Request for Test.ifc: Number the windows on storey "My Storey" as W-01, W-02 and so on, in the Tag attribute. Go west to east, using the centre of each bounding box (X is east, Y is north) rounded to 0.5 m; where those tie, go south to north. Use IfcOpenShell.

First a look at what the model holds.

```python
import ifcopenshell
import ifcopenshell.util.element
import ifcopenshell.util.placement

model = ifcopenshell.open("Test.ifc")
print(model.schema)
storey = next(s for s in model.by_type("IfcBuildingStorey") if s.Name == "My Storey")
windows = [e for e in ifcopenshell.util.element.get_decomposition(storey) if e.is_a("IfcWindow")]
for e in sorted(windows, key=lambda e: e.id()):
    origin = ifcopenshell.util.placement.get_local_placement(e.ObjectPlacement)[:3, 3]
    print(e.id(), e.Tag, e.Name, origin.round(2) + 0.0, sep=" | ")
```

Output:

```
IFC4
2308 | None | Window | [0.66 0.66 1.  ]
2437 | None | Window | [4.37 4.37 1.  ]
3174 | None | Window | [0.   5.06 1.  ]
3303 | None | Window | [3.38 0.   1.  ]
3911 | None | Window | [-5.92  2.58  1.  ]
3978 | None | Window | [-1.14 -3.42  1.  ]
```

```python
import ifcopenshell
import ifcopenshell.geom
import ifcopenshell.util.element
import ifcopenshell.util.shape

model = ifcopenshell.open("Test.ifc")
settings = ifcopenshell.geom.settings()
settings.set("use-world-coords", True)


def centre(element):
    shape = ifcopenshell.geom.create_shape(settings, element)
    return ifcopenshell.util.shape.get_bbox_centroid(shape.geometry)


storey = next(s for s in model.by_type("IfcBuildingStorey") if s.Name == "My Storey")
windows = [e for e in ifcopenshell.util.element.get_decomposition(storey) if e.is_a("IfcWindow")]

# Insertion points can sit at a corner or the storey origin, so sort by the geometry (in metres).
centres = {e: centre(e) for e in windows}
windows.sort(key=lambda e: (round(centres[e][0] / 0.5), centres[e][1]))

for i, e in enumerate(windows, start=1):
    number = f"W-{i:02d}"
    e.Tag = number
    print(e.id(), number)

model.write("Test_edited.ifc")
```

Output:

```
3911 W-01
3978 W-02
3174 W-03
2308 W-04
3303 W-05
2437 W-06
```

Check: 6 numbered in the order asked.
